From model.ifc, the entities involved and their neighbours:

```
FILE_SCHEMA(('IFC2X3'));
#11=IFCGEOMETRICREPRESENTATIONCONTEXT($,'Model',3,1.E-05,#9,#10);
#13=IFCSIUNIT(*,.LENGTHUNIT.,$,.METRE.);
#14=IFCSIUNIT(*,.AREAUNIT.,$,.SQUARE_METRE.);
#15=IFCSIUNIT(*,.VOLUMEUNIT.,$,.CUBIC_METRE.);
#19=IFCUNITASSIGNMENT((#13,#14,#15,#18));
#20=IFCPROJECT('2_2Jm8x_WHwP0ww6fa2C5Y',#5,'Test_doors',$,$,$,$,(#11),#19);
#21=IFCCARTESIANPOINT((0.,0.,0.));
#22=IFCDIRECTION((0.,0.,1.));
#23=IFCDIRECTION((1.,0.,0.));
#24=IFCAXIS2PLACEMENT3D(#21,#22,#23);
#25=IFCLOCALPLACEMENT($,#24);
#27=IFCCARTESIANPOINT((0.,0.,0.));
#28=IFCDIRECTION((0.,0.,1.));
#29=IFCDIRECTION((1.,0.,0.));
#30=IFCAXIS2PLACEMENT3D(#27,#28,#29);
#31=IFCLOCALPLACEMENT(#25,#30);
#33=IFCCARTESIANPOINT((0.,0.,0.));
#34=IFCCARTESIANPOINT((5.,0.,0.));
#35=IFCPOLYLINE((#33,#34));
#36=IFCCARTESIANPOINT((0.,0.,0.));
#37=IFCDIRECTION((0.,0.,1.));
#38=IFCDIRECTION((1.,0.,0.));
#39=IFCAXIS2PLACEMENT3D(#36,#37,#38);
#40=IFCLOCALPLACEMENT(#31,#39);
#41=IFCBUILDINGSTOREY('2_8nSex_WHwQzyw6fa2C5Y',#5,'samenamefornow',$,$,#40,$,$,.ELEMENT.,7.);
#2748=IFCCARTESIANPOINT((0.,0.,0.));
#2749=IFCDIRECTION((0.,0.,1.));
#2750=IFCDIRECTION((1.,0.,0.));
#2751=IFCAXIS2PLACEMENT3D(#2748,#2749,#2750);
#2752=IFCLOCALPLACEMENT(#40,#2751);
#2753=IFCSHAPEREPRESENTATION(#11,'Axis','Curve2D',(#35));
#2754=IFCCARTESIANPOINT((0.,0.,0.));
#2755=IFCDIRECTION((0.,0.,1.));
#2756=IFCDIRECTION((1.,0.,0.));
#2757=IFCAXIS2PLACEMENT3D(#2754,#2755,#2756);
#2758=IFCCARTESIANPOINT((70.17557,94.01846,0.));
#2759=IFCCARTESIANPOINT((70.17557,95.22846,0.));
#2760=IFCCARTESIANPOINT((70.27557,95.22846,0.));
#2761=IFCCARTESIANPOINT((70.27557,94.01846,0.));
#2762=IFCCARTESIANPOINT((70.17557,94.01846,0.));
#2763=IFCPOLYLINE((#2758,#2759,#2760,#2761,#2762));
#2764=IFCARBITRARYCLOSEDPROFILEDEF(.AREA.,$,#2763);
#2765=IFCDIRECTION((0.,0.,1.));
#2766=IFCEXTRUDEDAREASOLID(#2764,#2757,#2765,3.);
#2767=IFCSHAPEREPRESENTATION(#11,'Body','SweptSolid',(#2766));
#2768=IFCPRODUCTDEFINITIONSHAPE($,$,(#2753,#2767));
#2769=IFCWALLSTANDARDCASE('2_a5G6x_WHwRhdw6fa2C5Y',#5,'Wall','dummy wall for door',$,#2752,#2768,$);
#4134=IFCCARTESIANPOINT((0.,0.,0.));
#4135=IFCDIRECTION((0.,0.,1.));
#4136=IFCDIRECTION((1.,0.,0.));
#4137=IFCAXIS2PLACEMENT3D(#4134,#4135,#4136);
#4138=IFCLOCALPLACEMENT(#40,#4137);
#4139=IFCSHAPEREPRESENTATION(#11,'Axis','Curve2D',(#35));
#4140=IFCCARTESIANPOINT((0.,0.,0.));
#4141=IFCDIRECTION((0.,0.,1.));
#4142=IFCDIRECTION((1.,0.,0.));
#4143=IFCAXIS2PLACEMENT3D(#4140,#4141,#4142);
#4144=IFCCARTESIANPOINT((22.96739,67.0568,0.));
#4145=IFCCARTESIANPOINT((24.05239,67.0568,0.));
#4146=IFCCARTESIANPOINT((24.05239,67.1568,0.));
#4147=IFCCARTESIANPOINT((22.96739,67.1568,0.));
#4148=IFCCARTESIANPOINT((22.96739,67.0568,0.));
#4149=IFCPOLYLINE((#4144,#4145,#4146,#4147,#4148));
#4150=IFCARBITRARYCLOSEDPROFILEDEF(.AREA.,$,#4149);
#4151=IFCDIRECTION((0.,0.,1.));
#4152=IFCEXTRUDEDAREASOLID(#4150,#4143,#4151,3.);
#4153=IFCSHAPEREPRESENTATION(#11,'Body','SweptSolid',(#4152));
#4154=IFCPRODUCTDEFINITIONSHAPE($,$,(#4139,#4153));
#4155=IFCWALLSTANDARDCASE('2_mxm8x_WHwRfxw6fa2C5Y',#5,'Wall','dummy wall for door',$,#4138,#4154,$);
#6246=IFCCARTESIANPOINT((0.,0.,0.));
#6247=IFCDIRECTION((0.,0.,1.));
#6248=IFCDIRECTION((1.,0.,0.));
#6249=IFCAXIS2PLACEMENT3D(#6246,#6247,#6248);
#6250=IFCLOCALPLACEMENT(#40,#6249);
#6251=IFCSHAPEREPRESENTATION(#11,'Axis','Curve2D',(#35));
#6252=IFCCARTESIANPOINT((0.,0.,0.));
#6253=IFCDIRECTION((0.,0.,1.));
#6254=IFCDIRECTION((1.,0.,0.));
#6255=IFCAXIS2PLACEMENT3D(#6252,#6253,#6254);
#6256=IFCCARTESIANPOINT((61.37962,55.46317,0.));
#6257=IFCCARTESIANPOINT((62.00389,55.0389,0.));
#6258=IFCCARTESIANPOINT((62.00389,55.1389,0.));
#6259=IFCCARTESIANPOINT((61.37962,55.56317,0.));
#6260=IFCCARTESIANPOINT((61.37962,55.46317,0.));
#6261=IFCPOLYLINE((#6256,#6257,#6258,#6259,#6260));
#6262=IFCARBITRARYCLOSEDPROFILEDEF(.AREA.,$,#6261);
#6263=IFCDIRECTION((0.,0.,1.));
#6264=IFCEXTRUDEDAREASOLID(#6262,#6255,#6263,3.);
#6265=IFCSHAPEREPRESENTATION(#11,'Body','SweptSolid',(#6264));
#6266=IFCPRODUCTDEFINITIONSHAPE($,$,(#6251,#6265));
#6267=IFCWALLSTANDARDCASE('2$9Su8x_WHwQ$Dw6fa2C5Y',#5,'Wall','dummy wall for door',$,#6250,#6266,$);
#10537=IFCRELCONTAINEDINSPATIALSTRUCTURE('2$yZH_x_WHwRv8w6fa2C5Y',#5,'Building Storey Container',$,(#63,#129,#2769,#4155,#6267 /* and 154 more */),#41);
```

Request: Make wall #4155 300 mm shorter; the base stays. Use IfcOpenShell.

```python
import ifcopenshell
import ifcopenshell.geom
import ifcopenshell.util.shape
import ifcopenshell.util.unit

model = ifcopenshell.open("model.ifc")
unit_scale = ifcopenshell.util.unit.calculate_unit_scale(model)
settings = ifcopenshell.geom.settings()


def volume(element):
    """Net volume in cubic metres, openings subtracted."""
    shape = ifcopenshell.geom.create_shape(settings, element)
    return ifcopenshell.util.shape.get_volume(shape.geometry)


wall = model.by_guid("2_mxm8x_WHwRfxw6fa2C5Y")
before = volume(wall)

body = next(r for r in wall.Representation.Representations if r.RepresentationIdentifier == "Body")
solid = body.Items[0]
old_height = solid.Depth
solid.Depth -= 0.3 / unit_scale
after = volume(wall)

print(f"height {old_height:g} -> {solid.Depth:g}, volume {before:.3f} -> {after:.3f} m3")

model.write("model_updated.ifc")
```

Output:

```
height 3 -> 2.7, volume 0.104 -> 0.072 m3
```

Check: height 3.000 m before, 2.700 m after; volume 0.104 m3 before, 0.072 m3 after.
